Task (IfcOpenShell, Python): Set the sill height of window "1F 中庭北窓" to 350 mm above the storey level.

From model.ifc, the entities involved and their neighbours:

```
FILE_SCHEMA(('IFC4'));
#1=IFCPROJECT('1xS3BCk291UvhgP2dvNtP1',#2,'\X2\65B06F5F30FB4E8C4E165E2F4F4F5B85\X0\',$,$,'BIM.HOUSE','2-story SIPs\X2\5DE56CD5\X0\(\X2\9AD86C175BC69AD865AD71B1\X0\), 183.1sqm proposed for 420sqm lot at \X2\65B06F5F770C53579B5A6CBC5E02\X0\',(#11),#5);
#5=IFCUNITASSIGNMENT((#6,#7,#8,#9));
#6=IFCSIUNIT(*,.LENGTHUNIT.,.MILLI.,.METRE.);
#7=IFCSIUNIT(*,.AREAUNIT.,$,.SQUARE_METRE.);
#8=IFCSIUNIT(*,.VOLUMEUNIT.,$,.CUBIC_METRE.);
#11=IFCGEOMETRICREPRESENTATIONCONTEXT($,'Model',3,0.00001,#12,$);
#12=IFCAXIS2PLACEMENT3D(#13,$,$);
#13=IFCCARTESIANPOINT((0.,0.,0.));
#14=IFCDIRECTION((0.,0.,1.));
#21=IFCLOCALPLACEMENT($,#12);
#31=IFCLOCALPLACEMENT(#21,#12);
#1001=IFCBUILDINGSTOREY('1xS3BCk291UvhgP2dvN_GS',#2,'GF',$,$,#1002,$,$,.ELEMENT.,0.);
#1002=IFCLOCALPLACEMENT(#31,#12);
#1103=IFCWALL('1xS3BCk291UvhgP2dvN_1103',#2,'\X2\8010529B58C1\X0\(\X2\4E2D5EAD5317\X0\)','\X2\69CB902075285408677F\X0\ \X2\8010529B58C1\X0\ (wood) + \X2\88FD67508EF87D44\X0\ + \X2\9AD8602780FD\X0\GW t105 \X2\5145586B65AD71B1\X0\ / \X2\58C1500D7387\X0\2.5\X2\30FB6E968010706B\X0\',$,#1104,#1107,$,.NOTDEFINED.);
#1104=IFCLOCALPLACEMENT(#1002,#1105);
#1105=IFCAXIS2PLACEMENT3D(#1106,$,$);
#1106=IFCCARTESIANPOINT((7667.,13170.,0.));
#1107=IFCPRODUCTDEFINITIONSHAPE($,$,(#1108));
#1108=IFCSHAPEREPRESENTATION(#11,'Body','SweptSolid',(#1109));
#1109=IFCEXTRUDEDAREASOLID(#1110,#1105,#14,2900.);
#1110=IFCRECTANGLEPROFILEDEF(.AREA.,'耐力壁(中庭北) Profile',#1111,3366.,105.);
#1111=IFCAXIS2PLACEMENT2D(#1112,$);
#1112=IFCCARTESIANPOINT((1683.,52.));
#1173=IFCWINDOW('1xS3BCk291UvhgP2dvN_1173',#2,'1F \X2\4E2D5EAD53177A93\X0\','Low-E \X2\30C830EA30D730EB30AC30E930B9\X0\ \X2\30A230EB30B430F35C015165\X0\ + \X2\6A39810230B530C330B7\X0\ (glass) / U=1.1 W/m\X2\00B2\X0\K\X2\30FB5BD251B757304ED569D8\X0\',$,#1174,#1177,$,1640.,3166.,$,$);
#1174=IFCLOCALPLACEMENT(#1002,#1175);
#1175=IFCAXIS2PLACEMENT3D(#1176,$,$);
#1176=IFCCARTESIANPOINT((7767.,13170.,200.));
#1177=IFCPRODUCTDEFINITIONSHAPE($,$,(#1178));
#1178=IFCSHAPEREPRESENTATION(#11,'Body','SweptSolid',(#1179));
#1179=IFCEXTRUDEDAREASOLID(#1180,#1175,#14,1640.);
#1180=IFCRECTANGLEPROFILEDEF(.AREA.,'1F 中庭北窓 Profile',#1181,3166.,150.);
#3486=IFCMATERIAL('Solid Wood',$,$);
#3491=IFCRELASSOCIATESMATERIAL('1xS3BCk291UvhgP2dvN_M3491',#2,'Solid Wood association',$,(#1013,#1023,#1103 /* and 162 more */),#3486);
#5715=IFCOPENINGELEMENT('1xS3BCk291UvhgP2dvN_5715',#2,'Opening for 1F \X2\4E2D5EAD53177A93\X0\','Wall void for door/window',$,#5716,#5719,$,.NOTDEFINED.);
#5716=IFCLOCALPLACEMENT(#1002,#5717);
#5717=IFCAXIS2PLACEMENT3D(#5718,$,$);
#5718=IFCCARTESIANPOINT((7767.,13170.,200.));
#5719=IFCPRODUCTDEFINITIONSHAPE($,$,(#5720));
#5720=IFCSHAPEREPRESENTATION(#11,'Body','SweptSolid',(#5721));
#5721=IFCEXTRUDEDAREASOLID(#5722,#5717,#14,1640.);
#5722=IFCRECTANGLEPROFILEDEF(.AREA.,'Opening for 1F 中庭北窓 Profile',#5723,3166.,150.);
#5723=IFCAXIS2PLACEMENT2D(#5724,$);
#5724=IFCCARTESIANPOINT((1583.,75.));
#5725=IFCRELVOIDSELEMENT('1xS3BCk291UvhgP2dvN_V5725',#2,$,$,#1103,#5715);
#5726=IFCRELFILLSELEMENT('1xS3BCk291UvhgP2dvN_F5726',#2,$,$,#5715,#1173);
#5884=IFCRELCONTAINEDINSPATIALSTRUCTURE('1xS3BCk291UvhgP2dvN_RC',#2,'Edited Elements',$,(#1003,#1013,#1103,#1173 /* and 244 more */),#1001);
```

```python
import numpy as np
import ifcopenshell
import ifcopenshell.api.geometry
import ifcopenshell.geom
import ifcopenshell.util.element
import ifcopenshell.util.placement
import ifcopenshell.util.shape
import ifcopenshell.util.unit

model = ifcopenshell.open("model.ifc")
unit_scale = ifcopenshell.util.unit.calculate_unit_scale(model)

window = model.by_id(1173)
opening = window.FillsVoids[0].RelatingOpeningElement
storey = ifcopenshell.util.element.get_container(window, ifc_class="IfcBuildingStorey")
level = ifcopenshell.util.placement.get_local_placement(storey.ObjectPlacement)[2, 3]

# The opening's origin need not be at the sill, so measure its lowest point.
shape = ifcopenshell.geom.create_shape(ifcopenshell.geom.settings(), opening)
bottom = ifcopenshell.util.shape.get_shape_bottom_elevation(shape, shape.geometry) / unit_scale
dz = level + 0.35 / unit_scale - bottom

shift = np.array([0.0, 0.0, dz])
# The window is not placed relative to its opening, so move both.
for product in (opening, window):
    matrix = ifcopenshell.util.placement.get_local_placement(product.ObjectPlacement)
    matrix[:3, 3] += shift
    ifcopenshell.api.geometry.edit_object_placement(model, product=product, matrix=matrix, is_si=False)

print(f"moved by {dz * unit_scale:+.3f} m")

model.write("model_v2.ifc")
```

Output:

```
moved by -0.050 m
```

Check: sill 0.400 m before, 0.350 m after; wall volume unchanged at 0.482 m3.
